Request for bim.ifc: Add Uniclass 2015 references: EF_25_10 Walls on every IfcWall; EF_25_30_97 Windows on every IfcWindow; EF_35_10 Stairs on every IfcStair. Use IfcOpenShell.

First a look at what the model holds.

```python
import ifcopenshell

model = ifcopenshell.open("bim.ifc")
print(model.schema)
print("classifications:", [c.Name for c in model.by_type("IfcClassification")])
for ifc_class in ("IfcDoor", "IfcRoof", "IfcStair", "IfcWall", "IfcWindow"):
    print(ifc_class, len(model.by_type(ifc_class)))
```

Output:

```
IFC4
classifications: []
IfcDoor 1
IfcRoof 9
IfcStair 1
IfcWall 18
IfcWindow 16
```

```python
import ifcopenshell
import ifcopenshell.api.classification

model = ifcopenshell.open("bim.ifc")

system = ifcopenshell.api.classification.add_classification(model, classification="Uniclass 2015")

codes = {
    "IfcWall": ("EF_25_10", "Walls"),
    "IfcWindow": ("EF_25_30_97", "Windows"),
    "IfcStair": ("EF_35_10", "Stairs"),
}
for ifc_class, (code, name) in codes.items():
    products = model.by_type(ifc_class)
    ifcopenshell.api.classification.add_reference(
        model, products=products, classification=system, identification=code, name=name
    )
    print(code, len(products))

model.write("bim_rev.ifc")
```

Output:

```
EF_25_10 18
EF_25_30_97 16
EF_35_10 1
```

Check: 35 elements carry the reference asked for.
